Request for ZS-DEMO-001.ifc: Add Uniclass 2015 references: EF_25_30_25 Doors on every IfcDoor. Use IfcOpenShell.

First a look at what the model holds.

```python
import ifcopenshell

model = ifcopenshell.open("ZS-DEMO-001.ifc")
print(model.schema)
print("classifications:", [c.Name for c in model.by_type("IfcClassification")])
for ifc_class in ("IfcDoor", "IfcRoof", "IfcStair", "IfcWall", "IfcWindow"):
    print(ifc_class, len(model.by_type(ifc_class)))
```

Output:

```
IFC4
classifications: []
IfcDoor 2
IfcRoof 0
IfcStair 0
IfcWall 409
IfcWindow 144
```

```python
import ifcopenshell
import ifcopenshell.api.classification

model = ifcopenshell.open("ZS-DEMO-001.ifc")

system = ifcopenshell.api.classification.add_classification(model, classification="Uniclass 2015")

codes = {
    "IfcDoor": ("EF_25_30_25", "Doors"),
}
for ifc_class, (code, name) in codes.items():
    products = model.by_type(ifc_class)
    ifcopenshell.api.classification.add_reference(
        model, products=products, classification=system, identification=code, name=name
    )
    print(code, len(products))

model.write("ZS-DEMO-001_updated.ifc")
```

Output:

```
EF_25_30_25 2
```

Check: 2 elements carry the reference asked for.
